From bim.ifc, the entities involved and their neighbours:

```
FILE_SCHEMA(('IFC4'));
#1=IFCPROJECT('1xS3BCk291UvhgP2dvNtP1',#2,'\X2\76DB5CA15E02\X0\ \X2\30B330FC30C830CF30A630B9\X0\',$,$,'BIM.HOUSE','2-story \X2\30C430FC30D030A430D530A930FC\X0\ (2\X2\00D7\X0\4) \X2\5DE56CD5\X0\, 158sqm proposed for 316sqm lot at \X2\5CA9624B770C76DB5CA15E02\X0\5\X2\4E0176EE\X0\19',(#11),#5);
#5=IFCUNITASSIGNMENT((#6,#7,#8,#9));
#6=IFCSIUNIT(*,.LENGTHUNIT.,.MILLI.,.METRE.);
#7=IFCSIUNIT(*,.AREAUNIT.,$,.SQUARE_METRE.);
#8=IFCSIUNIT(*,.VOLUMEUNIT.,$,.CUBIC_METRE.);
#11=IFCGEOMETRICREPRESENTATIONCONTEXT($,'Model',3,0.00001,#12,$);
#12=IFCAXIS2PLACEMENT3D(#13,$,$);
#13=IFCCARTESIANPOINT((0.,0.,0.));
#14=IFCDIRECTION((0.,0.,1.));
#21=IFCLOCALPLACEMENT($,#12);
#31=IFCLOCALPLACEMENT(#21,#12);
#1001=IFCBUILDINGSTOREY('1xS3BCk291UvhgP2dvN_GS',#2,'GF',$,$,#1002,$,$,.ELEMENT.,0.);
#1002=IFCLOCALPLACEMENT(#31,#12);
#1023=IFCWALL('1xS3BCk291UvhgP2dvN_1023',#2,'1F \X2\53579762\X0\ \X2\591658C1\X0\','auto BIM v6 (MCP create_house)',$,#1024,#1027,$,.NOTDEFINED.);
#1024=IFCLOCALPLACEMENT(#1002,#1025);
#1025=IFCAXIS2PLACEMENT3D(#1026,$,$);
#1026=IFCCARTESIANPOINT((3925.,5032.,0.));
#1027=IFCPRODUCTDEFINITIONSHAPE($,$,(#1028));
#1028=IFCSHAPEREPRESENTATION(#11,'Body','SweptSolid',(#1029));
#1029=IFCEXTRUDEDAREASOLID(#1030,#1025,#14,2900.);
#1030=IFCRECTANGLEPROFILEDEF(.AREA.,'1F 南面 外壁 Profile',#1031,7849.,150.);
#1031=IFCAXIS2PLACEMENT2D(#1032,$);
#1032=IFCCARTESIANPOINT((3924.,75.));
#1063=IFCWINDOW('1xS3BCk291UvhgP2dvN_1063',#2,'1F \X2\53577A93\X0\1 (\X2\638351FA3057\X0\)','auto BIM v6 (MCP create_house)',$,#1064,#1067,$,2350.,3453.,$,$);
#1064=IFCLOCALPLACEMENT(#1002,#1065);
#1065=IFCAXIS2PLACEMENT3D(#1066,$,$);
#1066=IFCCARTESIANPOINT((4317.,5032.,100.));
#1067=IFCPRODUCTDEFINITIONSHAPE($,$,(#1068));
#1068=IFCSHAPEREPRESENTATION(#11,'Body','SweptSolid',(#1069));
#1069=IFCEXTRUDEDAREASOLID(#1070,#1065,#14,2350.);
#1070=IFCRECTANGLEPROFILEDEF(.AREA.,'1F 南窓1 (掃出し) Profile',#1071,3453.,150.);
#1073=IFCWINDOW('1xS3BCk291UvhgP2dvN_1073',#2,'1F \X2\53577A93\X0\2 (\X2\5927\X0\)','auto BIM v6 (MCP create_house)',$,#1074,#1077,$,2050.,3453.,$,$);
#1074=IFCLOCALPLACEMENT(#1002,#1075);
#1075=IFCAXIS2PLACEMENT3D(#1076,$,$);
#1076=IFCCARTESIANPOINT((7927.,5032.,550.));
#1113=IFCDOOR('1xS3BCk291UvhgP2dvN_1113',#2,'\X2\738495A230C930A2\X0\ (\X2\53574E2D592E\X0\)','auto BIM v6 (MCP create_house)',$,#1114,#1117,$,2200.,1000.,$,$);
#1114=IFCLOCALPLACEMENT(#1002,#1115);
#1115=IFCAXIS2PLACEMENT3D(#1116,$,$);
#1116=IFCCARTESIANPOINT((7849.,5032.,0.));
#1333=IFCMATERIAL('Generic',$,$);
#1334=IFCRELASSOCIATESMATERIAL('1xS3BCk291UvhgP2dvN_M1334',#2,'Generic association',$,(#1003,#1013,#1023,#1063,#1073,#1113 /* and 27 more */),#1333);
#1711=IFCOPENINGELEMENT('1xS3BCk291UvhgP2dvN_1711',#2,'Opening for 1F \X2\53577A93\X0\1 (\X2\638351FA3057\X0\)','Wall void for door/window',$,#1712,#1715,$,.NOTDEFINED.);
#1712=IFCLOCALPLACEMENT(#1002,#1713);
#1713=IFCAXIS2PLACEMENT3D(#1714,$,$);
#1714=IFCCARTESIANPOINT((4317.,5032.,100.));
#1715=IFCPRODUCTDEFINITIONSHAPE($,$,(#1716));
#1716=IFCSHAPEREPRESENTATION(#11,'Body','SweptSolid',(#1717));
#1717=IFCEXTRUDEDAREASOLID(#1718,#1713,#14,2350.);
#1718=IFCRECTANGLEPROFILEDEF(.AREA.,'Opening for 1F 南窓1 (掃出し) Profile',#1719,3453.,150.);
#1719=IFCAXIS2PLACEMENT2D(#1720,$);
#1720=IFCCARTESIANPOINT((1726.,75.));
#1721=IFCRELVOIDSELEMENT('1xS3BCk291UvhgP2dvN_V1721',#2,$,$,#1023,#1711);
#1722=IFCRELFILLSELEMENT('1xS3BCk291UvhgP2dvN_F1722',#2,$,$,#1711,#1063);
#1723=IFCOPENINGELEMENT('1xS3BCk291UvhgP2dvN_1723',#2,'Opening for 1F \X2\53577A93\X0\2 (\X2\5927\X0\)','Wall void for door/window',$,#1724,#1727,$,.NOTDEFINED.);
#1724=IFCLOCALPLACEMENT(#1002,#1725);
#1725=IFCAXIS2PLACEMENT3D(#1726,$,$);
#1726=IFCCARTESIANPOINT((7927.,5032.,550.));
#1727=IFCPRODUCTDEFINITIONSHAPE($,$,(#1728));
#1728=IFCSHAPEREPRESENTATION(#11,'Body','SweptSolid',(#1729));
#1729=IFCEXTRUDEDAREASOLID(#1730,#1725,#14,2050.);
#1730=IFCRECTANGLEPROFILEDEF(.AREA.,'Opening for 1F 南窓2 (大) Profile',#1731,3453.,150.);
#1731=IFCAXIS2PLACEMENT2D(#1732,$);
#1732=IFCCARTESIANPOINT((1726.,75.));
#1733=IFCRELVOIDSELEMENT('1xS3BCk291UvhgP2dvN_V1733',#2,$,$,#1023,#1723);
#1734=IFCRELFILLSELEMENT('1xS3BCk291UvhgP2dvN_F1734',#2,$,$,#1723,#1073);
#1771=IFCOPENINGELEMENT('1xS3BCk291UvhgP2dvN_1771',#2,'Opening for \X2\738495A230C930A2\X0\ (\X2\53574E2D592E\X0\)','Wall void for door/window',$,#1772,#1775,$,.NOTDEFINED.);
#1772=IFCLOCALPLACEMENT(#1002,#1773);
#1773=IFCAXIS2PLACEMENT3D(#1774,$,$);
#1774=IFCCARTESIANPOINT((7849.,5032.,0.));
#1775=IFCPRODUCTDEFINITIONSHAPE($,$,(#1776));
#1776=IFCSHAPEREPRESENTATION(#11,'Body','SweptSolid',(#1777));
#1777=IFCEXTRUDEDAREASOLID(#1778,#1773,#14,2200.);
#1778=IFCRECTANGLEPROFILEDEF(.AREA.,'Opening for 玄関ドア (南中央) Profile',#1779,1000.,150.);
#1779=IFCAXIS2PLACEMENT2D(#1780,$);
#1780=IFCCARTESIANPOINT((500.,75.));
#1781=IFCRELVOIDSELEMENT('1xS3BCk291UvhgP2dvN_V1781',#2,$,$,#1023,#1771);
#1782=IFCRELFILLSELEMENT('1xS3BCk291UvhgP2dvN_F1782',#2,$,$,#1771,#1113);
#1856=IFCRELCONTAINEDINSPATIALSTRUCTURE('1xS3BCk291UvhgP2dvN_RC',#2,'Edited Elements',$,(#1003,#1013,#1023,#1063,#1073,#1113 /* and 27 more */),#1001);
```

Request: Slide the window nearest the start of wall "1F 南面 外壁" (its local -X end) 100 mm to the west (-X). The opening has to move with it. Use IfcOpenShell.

```python
import ifcopenshell
import ifcopenshell.api.geometry
import ifcopenshell.util.placement

model = ifcopenshell.open("bim.ifc")

window = model.by_guid("1xS3BCk291UvhgP2dvN_1063")
opening = window.FillsVoids[0].RelatingOpeningElement
wall = opening.VoidsElements[0].RelatingBuildingElement

wall_matrix = ifcopenshell.util.placement.get_local_placement(wall.ObjectPlacement)
shift = wall_matrix[:3, 0] * -100.0
before = ifcopenshell.util.placement.get_local_placement(window.ObjectPlacement)[:3, 3].copy()

# The window is not placed relative to its opening, so move both.
for product in (opening, window):
    matrix = ifcopenshell.util.placement.get_local_placement(product.ObjectPlacement)
    matrix[:3, 3] += shift
    ifcopenshell.api.geometry.edit_object_placement(model, product=product, matrix=matrix, is_si=False)

after = ifcopenshell.util.placement.get_local_placement(window.ObjectPlacement)[:3, 3]
print("window moved by", (after - before).round(3) + 0.0)

model.write("bim_rev.ifc")
```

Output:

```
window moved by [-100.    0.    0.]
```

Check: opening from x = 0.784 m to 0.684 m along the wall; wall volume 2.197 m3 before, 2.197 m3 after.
